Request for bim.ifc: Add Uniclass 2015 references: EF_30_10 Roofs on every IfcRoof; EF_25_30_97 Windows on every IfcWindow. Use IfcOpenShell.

First a look at what the model holds.

```python
import ifcopenshell

model = ifcopenshell.open("bim.ifc")
print(model.schema)
print("classifications:", [c.Name for c in model.by_type("IfcClassification")])
for ifc_class in ("IfcDoor", "IfcRoof", "IfcStair", "IfcWall", "IfcWindow"):
    print(ifc_class, len(model.by_type(ifc_class)))
```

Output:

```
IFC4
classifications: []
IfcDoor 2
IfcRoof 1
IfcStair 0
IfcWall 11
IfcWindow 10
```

```python
import ifcopenshell
import ifcopenshell.api.classification

model = ifcopenshell.open("bim.ifc")

system = ifcopenshell.api.classification.add_classification(model, classification="Uniclass 2015")

codes = {
    "IfcRoof": ("EF_30_10", "Roofs"),
    "IfcWindow": ("EF_25_30_97", "Windows"),
}
for ifc_class, (code, name) in codes.items():
    products = model.by_type(ifc_class)
    ifcopenshell.api.classification.add_reference(
        model, products=products, classification=system, identification=code, name=name
    )
    print(code, len(products))

model.write("bim_edited.ifc")
```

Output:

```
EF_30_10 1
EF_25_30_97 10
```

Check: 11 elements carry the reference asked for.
